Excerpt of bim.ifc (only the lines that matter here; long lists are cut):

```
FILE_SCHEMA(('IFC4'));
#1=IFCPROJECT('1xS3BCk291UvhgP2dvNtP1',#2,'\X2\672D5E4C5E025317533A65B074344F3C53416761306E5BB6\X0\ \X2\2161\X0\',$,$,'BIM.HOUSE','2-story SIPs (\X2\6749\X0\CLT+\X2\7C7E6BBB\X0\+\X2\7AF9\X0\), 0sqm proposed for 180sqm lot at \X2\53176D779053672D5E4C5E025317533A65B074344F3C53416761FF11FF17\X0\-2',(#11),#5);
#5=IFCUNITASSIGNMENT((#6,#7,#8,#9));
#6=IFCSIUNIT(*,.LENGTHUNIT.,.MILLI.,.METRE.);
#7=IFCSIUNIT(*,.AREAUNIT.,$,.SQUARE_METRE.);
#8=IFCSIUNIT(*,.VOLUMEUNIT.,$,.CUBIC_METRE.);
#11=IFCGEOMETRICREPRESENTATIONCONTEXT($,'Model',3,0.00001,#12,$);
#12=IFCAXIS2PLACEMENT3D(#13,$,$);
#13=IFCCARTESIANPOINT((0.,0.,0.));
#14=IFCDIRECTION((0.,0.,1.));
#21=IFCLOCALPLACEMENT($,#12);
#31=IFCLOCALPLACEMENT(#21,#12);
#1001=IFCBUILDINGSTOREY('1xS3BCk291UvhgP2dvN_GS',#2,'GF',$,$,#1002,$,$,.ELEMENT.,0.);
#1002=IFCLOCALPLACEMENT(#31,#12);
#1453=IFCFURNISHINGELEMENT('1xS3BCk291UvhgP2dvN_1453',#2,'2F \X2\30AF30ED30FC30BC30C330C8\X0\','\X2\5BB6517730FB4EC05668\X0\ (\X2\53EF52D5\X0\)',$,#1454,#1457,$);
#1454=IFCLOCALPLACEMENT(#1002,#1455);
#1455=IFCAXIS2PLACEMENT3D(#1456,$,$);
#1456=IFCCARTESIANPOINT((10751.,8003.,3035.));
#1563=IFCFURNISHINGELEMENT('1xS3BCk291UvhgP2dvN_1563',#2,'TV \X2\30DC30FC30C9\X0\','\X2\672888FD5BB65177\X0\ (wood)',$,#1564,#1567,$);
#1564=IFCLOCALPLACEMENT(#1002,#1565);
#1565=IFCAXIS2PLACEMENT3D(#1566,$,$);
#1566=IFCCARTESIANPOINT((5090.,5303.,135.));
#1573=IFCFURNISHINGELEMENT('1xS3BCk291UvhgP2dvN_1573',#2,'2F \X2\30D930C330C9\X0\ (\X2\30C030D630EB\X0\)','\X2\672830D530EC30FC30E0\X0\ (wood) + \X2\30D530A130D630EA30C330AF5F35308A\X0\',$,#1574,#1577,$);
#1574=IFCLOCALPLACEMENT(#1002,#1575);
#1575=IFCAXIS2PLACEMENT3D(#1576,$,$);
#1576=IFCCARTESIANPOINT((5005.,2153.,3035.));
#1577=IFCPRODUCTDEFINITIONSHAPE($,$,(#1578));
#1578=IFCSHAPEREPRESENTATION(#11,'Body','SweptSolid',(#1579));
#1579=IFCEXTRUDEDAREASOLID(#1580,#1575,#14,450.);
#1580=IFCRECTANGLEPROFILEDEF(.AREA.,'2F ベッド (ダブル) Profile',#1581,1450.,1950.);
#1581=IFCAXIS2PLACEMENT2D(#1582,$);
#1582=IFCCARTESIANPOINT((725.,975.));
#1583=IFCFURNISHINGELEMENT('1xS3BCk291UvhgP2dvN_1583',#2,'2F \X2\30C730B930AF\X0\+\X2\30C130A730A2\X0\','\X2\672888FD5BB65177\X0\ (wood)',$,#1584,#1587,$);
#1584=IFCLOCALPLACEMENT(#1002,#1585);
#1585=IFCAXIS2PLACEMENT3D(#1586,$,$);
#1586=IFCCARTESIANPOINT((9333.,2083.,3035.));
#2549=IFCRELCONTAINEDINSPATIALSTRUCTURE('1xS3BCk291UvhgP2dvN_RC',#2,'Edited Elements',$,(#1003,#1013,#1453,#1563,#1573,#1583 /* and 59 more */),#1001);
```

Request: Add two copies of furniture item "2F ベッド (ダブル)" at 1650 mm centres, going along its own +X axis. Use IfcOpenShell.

```python
import ifcopenshell
import ifcopenshell.api.geometry
import ifcopenshell.api.root
import ifcopenshell.util.element
import ifcopenshell.util.placement

model = ifcopenshell.open("bim.ifc")


def reuse_history(source, copy):
    """copy_class also copies each property set's owner history, people and application; keep the originals."""
    for rel in copy.IsDefinedBy:
        if rel.is_a("IfcRelDefinesByProperties") and (history := rel.RelatingPropertyDefinition.OwnerHistory):
            rel.RelatingPropertyDefinition.OwnerHistory = source.OwnerHistory
            ifcopenshell.util.element.remove_deep2(model, history)


source = model.by_guid("1xS3BCk291UvhgP2dvN_1573")
base = ifcopenshell.util.placement.get_local_placement(source.ObjectPlacement)
step = base[:3, 0] * 1650.0

for i in range(1, 3):
    copy = ifcopenshell.api.root.copy_class(model, product=source)
    copy.Representation = ifcopenshell.util.element.copy_deep(
        model, source.Representation, exclude=["IfcGeometricRepresentationContext", "IfcRepresentationMap"]
    )
    reuse_history(source, copy)
    matrix = base.copy()
    matrix[:3, 3] += i * step
    print("added at", matrix[:3, 3].round(3) + 0.0)
    ifcopenshell.api.geometry.edit_object_placement(model, product=copy, matrix=matrix, is_si=False)

model.write("bim-out.ifc")
```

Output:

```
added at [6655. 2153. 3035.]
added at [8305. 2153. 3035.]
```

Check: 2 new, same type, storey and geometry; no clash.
